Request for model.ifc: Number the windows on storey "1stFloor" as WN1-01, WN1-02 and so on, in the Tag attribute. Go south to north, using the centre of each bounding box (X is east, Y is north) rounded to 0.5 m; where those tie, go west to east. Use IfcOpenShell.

First a look at what the model holds.

```python
import ifcopenshell
import ifcopenshell.util.element
import ifcopenshell.util.placement

model = ifcopenshell.open("model.ifc")
print(model.schema)
storey = next(s for s in model.by_type("IfcBuildingStorey") if s.Name == "1stFloor")
windows = [e for e in ifcopenshell.util.element.get_decomposition(storey) if e.is_a("IfcWindow")]
for e in sorted(windows, key=lambda e: e.id()):
    origin = ifcopenshell.util.placement.get_local_placement(e.ObjectPlacement)[:3, 3]
    print(e.id(), e.Tag, e.Name, origin.round(2) + 0.0, sep=" | ")
```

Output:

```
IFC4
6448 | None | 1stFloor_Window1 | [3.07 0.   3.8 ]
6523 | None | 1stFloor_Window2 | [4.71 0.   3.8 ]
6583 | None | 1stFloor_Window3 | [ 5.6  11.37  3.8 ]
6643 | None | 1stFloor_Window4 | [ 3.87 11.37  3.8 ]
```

```python
import ifcopenshell
import ifcopenshell.geom
import ifcopenshell.util.element
import ifcopenshell.util.shape

model = ifcopenshell.open("model.ifc")
settings = ifcopenshell.geom.settings()
settings.set("use-world-coords", True)


def centre(element):
    shape = ifcopenshell.geom.create_shape(settings, element)
    return ifcopenshell.util.shape.get_bbox_centroid(shape.geometry)


storey = next(s for s in model.by_type("IfcBuildingStorey") if s.Name == "1stFloor")
windows = [e for e in ifcopenshell.util.element.get_decomposition(storey) if e.is_a("IfcWindow")]

# Insertion points can sit at a corner or the storey origin, so sort by the geometry (in metres).
centres = {e: centre(e) for e in windows}
windows.sort(key=lambda e: (round(centres[e][1] / 0.5), centres[e][0]))

for i, e in enumerate(windows, start=1):
    number = f"WN1-{i:02d}"
    e.Tag = number
    print(e.id(), number)

model.write("model_v2.ifc")
```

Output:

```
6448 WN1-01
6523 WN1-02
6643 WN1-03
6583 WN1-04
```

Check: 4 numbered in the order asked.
